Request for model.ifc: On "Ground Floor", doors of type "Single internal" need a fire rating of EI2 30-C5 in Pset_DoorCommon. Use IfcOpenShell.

First a look at what the model holds.

```python
import ifcopenshell
import ifcopenshell.util.element

model = ifcopenshell.open("model.ifc")
print(model.schema)
storey = next(s for s in model.by_type("IfcBuildingStorey") if s.Name == "Ground Floor")
doors = [e for e in ifcopenshell.util.element.get_decomposition(storey) if e.is_a("IfcDoor")]
seen = {}
for e in doors:
    element_type = ifcopenshell.util.element.get_type(e)
    key = (element_type.Name if element_type != e and element_type else None, ifcopenshell.util.element.get_pset(e, "Pset_DoorCommon", "FireRating"))
    seen[key] = seen.get(key, 0) + 1
for (name, value), count in sorted(seen.items(), key=str):
    print(count, "x", name, "|", value)
```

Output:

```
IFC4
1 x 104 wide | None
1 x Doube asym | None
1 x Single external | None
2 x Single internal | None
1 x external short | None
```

```python
import ifcopenshell
import ifcopenshell.api.pset
import ifcopenshell.util.element

model = ifcopenshell.open("model.ifc")

storey = next(s for s in model.by_type("IfcBuildingStorey") if s.Name == "Ground Floor")
doors = [e for e in ifcopenshell.util.element.get_decomposition(storey) if e.is_a("IfcDoor")]

count = 0
for e in doors:
    element_type = ifcopenshell.util.element.get_type(e)
    if element_type in (None, e) or element_type.Name != "Single internal":
        continue
    # add_pset returns the element's existing set when there is one.
    pset = ifcopenshell.api.pset.add_pset(model, product=e, name="Pset_DoorCommon")
    ifcopenshell.api.pset.edit_pset(model, pset=pset, properties={"FireRating": "EI2 30-C5"})
    count += 1

print(count, "doors updated")

model.write("model_v2.ifc")
```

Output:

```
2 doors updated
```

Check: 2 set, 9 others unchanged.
